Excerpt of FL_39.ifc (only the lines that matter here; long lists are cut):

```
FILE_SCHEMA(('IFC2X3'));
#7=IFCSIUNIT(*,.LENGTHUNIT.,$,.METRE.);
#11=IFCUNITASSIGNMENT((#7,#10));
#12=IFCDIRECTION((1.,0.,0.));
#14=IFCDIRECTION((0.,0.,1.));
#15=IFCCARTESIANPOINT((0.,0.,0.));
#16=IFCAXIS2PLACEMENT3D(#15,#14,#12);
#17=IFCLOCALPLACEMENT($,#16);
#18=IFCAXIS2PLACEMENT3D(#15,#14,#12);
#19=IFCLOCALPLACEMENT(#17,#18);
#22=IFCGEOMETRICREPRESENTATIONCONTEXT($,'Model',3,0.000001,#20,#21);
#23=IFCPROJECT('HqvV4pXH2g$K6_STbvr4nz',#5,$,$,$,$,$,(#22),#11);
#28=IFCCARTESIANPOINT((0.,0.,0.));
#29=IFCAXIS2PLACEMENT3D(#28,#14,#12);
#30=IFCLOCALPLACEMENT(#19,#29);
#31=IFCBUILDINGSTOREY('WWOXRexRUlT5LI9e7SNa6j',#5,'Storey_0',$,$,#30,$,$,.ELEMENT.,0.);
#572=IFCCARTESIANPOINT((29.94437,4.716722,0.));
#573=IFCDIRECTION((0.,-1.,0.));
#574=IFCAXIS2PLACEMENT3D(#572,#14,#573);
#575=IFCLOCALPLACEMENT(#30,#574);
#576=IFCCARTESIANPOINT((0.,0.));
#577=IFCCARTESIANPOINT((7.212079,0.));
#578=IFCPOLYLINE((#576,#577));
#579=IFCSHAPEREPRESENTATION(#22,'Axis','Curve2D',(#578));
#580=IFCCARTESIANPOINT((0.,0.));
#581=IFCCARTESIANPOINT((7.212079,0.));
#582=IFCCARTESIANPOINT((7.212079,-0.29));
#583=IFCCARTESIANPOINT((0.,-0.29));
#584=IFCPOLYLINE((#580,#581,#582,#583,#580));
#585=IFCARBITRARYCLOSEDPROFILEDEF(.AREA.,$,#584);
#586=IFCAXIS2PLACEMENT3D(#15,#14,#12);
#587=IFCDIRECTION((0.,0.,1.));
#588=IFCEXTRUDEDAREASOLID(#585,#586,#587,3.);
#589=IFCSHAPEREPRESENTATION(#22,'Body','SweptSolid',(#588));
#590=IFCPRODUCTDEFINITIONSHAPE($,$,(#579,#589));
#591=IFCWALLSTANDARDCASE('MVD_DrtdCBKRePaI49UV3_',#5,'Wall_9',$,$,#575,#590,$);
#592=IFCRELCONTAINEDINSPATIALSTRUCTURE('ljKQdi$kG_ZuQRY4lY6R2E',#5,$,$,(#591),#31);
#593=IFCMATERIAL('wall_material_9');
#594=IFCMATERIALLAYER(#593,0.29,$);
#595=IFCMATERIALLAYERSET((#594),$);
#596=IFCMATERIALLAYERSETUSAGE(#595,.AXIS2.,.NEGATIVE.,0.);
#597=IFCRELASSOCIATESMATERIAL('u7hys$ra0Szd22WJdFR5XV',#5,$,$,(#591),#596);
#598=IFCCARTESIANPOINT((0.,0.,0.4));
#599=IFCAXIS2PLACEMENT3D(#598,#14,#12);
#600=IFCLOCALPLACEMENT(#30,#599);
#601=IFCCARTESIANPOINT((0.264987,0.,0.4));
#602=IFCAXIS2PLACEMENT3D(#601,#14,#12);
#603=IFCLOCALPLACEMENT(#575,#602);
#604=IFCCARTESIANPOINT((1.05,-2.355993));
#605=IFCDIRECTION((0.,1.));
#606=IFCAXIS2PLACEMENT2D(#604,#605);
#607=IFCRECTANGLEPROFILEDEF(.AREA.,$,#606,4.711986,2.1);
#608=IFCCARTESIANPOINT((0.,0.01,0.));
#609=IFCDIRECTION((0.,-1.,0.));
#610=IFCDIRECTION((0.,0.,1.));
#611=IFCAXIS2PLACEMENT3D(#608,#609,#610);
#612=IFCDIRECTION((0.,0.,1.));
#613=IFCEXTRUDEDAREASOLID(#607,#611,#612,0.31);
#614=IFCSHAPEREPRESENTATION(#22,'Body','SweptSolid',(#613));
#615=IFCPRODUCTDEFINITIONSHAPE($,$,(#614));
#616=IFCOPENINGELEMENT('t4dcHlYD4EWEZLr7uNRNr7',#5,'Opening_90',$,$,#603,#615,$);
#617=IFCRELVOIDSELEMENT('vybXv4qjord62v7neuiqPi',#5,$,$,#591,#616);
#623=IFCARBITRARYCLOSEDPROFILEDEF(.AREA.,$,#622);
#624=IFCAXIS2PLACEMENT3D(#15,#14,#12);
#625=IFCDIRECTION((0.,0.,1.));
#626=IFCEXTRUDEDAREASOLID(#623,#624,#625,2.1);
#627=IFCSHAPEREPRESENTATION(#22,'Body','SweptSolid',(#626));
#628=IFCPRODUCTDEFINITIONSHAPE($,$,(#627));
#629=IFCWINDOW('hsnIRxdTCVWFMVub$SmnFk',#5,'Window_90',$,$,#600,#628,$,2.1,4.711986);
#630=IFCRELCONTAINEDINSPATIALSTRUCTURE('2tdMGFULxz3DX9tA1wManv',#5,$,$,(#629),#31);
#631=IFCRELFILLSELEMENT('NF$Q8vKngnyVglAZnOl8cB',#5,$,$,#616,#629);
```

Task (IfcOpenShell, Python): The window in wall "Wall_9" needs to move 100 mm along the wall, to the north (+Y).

```python
import ifcopenshell
import ifcopenshell.api.geometry
import ifcopenshell.util.placement

model = ifcopenshell.open("FL_39.ifc")

window = model.by_guid("hsnIRxdTCVWFMVub$SmnFk")
opening = window.FillsVoids[0].RelatingOpeningElement
wall = opening.VoidsElements[0].RelatingBuildingElement

wall_matrix = ifcopenshell.util.placement.get_local_placement(wall.ObjectPlacement)
shift = wall_matrix[:3, 0] * -0.1
before = ifcopenshell.util.placement.get_local_placement(window.ObjectPlacement)[:3, 3].copy()

# The window is not placed relative to its opening, so move both.
for product in (opening, window):
    matrix = ifcopenshell.util.placement.get_local_placement(product.ObjectPlacement)
    matrix[:3, 3] += shift
    ifcopenshell.api.geometry.edit_object_placement(model, product=product, matrix=matrix, is_si=False)

after = ifcopenshell.util.placement.get_local_placement(window.ObjectPlacement)[:3, 3]
print("window moved by", (after - before).round(3) + 0.0)

model.write("FL_39-out.ifc")
```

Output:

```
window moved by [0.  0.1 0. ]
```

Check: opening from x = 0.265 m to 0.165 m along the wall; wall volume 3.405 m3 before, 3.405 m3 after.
